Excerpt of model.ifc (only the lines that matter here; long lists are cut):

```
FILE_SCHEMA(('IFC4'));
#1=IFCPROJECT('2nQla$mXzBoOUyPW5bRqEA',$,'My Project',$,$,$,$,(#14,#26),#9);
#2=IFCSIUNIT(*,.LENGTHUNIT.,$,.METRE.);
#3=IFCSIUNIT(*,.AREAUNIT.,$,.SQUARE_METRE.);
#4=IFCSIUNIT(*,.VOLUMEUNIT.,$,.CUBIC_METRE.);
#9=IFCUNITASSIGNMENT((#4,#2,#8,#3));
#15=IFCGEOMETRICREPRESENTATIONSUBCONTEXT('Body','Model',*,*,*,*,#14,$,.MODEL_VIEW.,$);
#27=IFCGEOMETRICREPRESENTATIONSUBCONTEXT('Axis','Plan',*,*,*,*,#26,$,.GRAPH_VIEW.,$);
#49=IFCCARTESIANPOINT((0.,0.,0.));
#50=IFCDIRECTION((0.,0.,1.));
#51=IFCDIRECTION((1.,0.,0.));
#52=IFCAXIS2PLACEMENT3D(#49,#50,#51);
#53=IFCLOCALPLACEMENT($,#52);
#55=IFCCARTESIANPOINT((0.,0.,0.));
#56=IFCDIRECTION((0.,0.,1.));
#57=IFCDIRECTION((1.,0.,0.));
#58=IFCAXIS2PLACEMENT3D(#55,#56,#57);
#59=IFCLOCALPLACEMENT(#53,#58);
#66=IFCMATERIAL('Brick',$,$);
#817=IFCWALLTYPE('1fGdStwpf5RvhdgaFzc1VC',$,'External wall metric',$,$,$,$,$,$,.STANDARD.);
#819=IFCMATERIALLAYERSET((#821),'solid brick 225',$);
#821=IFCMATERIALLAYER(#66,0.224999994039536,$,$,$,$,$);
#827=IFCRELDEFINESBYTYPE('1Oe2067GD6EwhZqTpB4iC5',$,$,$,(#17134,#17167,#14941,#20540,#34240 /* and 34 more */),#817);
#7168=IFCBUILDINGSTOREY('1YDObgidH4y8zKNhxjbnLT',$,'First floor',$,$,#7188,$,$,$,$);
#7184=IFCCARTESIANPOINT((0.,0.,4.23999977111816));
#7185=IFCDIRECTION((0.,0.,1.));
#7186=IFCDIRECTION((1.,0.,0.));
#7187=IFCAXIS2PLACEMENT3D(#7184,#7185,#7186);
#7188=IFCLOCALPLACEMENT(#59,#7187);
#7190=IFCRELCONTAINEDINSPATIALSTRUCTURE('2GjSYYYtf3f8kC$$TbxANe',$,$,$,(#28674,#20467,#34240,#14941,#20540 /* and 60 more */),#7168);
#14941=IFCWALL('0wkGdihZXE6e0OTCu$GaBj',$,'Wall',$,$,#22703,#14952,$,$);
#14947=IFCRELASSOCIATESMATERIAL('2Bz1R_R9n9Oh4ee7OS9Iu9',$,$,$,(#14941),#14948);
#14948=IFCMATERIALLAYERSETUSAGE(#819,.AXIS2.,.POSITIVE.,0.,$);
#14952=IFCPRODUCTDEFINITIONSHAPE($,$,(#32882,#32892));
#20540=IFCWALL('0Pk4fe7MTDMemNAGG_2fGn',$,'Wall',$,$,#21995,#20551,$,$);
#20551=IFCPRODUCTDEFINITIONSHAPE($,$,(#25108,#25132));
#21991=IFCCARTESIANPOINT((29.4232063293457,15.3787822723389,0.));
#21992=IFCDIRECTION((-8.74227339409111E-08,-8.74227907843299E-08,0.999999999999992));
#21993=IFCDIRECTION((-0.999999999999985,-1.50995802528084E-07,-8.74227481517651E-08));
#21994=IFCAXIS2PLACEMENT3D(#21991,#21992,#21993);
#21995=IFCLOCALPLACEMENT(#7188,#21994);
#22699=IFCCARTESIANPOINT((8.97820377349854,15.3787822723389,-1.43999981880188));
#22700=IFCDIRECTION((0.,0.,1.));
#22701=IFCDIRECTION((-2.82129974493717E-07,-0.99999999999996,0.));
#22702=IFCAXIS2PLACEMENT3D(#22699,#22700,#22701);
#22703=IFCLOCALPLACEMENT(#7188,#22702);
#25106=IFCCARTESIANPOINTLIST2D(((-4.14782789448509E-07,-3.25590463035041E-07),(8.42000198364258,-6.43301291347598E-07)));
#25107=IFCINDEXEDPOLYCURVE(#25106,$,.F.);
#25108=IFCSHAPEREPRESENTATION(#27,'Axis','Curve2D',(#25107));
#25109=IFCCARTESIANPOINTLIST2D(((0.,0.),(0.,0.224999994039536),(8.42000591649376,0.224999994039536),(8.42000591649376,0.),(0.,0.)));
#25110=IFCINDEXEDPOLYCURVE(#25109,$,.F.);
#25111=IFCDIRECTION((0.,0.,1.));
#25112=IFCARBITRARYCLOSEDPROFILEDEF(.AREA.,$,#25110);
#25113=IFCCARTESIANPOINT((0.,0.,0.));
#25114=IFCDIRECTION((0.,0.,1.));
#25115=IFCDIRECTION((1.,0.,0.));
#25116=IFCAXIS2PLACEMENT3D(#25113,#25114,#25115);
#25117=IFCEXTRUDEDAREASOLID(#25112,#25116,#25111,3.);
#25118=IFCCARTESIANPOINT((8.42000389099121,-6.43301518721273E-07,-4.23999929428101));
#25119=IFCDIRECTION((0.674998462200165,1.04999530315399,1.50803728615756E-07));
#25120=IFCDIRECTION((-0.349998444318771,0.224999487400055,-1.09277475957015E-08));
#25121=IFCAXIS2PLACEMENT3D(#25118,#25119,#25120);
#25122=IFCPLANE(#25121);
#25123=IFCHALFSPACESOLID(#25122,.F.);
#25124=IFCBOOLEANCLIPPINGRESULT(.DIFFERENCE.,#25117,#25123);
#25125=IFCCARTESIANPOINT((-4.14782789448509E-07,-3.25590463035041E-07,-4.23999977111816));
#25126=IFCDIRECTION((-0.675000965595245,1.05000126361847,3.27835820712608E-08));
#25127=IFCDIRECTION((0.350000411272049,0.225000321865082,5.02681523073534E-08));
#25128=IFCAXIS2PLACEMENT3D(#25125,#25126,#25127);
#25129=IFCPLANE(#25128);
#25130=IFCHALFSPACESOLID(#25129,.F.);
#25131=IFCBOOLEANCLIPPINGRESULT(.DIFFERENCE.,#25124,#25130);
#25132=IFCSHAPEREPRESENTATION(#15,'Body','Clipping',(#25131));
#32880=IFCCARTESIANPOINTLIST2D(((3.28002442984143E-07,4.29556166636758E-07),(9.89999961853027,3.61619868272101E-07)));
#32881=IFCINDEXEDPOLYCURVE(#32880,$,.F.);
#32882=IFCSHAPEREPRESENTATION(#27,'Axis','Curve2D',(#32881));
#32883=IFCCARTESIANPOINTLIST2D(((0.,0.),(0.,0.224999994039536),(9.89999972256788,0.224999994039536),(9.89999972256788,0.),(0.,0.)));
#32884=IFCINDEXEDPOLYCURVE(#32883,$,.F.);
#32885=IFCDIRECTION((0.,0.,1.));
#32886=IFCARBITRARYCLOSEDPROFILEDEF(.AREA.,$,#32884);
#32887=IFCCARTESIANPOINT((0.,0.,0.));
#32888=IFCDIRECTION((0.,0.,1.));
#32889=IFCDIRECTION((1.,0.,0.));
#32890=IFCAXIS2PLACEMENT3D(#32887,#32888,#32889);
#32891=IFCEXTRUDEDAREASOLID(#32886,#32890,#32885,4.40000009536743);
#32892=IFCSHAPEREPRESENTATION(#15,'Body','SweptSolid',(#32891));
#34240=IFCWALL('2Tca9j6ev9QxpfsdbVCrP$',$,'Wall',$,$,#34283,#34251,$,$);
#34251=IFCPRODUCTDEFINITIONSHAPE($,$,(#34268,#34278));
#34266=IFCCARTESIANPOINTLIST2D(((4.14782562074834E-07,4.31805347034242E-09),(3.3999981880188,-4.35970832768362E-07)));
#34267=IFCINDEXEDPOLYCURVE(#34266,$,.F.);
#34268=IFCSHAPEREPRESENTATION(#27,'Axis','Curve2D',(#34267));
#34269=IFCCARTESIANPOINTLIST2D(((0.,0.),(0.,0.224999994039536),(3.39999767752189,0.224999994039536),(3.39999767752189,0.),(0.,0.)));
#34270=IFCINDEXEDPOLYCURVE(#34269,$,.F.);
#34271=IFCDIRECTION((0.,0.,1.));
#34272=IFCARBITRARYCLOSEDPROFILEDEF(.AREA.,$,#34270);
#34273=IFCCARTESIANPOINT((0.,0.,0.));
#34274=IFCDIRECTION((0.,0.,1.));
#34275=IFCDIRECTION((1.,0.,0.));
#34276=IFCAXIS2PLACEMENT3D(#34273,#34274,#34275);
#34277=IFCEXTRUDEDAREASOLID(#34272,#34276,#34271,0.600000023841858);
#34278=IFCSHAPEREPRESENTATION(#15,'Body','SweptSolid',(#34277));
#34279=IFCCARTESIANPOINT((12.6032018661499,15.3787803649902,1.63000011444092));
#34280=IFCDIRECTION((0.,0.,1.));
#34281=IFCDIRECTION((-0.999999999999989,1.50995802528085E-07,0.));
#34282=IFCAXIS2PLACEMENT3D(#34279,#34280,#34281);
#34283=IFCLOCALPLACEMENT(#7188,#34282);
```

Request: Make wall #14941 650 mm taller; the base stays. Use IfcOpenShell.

```python
import ifcopenshell
import ifcopenshell.geom
import ifcopenshell.util.representation
import ifcopenshell.util.shape

model = ifcopenshell.open("model.ifc")
settings = ifcopenshell.geom.settings()


def volume(element):
    """Net volume in cubic metres, openings subtracted."""
    shape = ifcopenshell.geom.create_shape(settings, element)
    return ifcopenshell.util.shape.get_volume(shape.geometry)


wall = model.by_guid("0wkGdihZXE6e0OTCu$GaBj")
before = volume(wall)

body = ifcopenshell.util.representation.get_representation(wall, "Model", "Body")
solid = body.Items[0]
old_height = solid.Depth
solid.Depth += 0.65
after = volume(wall)

print(f"height {old_height:g} -> {solid.Depth:g}, volume {before:.3f} -> {after:.3f} m3")

model.write("model_edited.ifc")
```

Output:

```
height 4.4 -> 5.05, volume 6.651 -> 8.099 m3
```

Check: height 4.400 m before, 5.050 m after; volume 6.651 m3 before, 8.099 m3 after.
